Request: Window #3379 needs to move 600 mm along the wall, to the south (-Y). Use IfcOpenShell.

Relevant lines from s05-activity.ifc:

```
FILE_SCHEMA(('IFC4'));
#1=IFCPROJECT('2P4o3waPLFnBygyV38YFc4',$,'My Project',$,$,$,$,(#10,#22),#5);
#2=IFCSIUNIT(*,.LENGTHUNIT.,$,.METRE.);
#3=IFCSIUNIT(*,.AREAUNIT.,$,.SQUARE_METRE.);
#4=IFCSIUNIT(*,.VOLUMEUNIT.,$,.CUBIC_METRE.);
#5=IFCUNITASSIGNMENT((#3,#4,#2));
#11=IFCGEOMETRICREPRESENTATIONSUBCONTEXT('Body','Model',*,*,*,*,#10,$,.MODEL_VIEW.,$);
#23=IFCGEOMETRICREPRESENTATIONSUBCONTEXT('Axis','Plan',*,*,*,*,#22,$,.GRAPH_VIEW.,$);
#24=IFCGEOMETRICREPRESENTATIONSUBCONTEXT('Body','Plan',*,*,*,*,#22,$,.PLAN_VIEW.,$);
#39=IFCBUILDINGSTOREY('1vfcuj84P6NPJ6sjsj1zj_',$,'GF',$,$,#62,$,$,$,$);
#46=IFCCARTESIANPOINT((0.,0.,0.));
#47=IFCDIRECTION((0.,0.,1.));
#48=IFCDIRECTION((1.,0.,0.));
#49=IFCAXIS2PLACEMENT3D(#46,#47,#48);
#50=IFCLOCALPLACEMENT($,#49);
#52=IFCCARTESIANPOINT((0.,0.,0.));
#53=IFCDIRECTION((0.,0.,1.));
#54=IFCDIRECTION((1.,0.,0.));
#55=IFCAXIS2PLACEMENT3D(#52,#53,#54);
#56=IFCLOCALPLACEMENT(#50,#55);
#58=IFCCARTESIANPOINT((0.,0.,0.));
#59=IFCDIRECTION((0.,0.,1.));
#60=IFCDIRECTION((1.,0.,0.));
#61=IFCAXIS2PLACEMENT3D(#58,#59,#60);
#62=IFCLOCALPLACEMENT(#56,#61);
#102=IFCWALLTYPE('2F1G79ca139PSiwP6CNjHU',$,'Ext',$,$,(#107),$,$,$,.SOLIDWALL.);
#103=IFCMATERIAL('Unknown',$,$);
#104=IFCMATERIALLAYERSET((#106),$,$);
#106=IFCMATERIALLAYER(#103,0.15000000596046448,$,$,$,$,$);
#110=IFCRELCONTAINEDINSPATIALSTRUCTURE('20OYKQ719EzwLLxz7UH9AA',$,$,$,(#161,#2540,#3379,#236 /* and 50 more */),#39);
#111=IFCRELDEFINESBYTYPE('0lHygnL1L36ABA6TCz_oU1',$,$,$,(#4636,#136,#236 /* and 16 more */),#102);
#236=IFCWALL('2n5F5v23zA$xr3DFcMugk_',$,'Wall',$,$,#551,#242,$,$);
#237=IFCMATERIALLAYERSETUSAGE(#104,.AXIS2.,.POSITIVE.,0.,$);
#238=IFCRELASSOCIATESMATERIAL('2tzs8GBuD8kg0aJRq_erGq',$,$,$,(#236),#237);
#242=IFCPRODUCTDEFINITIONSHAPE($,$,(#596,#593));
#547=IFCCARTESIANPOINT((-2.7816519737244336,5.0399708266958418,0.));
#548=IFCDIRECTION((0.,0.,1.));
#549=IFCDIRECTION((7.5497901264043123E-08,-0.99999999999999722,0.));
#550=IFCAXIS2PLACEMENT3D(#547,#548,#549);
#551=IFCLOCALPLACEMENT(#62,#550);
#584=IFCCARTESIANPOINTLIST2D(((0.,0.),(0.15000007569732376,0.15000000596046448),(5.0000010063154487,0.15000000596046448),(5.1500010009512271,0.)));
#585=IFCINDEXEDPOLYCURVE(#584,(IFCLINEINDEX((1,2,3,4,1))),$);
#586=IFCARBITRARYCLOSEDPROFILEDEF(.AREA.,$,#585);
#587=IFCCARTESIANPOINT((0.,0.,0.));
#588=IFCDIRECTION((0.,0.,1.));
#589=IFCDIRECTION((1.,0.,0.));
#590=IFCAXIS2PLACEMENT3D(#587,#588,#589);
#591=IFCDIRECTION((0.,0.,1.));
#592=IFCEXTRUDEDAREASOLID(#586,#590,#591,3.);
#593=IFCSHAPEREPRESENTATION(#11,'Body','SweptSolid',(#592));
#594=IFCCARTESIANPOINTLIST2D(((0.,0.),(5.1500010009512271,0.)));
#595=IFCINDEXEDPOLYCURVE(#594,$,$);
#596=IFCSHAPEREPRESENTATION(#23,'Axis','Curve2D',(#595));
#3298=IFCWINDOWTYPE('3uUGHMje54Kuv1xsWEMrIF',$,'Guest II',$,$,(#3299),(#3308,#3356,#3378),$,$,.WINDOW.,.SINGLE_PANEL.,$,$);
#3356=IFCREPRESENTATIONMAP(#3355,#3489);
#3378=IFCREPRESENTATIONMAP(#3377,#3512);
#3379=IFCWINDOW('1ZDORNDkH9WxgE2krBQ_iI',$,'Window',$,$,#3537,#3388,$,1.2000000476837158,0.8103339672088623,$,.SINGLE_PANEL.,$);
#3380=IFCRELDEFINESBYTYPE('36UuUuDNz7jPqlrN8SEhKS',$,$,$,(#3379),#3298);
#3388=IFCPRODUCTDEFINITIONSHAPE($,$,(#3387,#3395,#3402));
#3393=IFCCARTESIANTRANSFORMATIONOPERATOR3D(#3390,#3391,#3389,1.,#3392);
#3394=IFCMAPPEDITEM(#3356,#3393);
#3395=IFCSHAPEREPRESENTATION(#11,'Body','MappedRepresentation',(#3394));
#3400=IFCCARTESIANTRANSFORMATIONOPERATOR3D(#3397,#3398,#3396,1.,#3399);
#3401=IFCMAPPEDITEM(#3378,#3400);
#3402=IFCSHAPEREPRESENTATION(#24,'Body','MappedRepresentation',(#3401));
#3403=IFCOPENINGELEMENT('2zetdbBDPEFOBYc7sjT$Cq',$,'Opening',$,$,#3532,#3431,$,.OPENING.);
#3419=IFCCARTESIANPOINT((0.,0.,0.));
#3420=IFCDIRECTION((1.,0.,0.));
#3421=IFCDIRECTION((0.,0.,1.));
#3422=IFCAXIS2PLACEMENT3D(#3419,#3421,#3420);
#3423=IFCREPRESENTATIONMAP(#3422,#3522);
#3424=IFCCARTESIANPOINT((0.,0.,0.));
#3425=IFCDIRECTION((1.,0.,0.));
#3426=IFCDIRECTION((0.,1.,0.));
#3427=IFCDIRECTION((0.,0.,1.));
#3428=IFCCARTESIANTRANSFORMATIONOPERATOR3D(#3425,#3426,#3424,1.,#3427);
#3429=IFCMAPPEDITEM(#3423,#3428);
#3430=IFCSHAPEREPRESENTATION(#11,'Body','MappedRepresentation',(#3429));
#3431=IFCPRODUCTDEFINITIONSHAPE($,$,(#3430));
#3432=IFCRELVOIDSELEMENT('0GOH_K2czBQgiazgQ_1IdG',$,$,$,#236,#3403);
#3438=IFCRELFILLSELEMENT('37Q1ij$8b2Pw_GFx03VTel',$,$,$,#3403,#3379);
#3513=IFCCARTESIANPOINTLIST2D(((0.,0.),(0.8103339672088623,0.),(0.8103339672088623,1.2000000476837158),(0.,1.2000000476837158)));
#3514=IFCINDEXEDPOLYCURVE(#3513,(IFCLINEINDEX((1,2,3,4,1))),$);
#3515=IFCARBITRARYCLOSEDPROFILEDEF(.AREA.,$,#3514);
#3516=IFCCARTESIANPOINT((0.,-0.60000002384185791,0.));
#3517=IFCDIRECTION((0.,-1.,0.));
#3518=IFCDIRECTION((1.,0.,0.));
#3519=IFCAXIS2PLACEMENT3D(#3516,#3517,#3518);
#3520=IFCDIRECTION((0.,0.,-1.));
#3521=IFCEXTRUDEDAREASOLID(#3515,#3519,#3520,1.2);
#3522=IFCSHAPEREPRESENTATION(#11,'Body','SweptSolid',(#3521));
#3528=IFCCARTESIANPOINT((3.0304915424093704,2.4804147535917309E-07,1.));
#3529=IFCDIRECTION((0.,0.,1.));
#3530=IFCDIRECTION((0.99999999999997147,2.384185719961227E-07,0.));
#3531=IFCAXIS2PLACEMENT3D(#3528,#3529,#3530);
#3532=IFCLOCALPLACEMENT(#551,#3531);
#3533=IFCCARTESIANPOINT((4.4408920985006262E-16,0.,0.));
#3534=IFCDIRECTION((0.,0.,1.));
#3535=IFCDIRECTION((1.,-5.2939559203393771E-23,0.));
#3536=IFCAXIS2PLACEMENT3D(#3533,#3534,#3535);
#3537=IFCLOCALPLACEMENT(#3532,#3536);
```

```python
import ifcopenshell
import ifcopenshell.api.geometry
import ifcopenshell.util.placement

model = ifcopenshell.open("s05-activity.ifc")

window = model.by_id(3379)
opening = window.FillsVoids[0].RelatingOpeningElement
wall = opening.VoidsElements[0].RelatingBuildingElement

wall_matrix = ifcopenshell.util.placement.get_local_placement(wall.ObjectPlacement)
shift = wall_matrix[:3, 0] * 0.6
before = ifcopenshell.util.placement.get_local_placement(window.ObjectPlacement)[:3, 3].copy()

# The window is placed relative to its opening, so it follows when the opening moves.
matrix = ifcopenshell.util.placement.get_local_placement(opening.ObjectPlacement)
matrix[:3, 3] += shift
ifcopenshell.api.geometry.edit_object_placement(
    model, product=opening, matrix=matrix, is_si=False, should_transform_children=True
)

after = ifcopenshell.util.placement.get_local_placement(window.ObjectPlacement)[:3, 3]
print("window moved by", (after - before).round(3) + 0.0)

model.write("s05-activity_edited.ifc")
```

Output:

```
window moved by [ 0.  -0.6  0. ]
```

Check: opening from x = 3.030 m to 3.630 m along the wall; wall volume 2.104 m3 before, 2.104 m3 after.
